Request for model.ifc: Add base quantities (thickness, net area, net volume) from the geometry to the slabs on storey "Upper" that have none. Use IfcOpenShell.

First a look at what the model holds.

```python
import ifcopenshell
import ifcopenshell.util.element
import ifcopenshell.util.unit

model = ifcopenshell.open("model.ifc")
print(model.schema)
for unit_type in ("LENGTHUNIT", "AREAUNIT", "VOLUMEUNIT"):
    print(unit_type, ifcopenshell.util.unit.calculate_unit_scale(model, unit_type))
storey = next(s for s in model.by_type("IfcBuildingStorey") if s.Name == "Upper")
slabs = [e for e in ifcopenshell.util.element.get_decomposition(storey) if e.is_a("IfcSlab")]
for e in sorted(slabs, key=lambda e: e.id()):
    print(e.id(), e.is_a(), e.Name, list(ifcopenshell.util.element.get_psets(e, qtos_only=True)), sep=" | ")
```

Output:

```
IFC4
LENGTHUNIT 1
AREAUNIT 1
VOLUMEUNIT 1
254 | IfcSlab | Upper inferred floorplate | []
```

```python
import ifcopenshell
import ifcopenshell.api.pset
import ifcopenshell.geom
import ifcopenshell.util.element
import ifcopenshell.util.shape
import ifcopenshell.util.unit

model = ifcopenshell.open("model.ifc")
unit_scale = ifcopenshell.util.unit.calculate_unit_scale(model)
area_scale = ifcopenshell.util.unit.calculate_unit_scale(model, "AREAUNIT")
volume_scale = ifcopenshell.util.unit.calculate_unit_scale(model, "VOLUMEUNIT")
settings = ifcopenshell.geom.settings()

storey = next(s for s in model.by_type("IfcBuildingStorey") if s.Name == "Upper")
slabs = [e for e in ifcopenshell.util.element.get_decomposition(storey) if e.is_a("IfcSlab")]

for e in sorted(slabs, key=lambda e: e.id()):
    if ifcopenshell.util.element.get_psets(e, qtos_only=True, should_inherit=False):
        continue
    # Geometry comes back in metres, in the element's own axes.
    shape = ifcopenshell.geom.create_shape(settings, e)
    values = {
        "Width": ifcopenshell.util.shape.get_z(shape.geometry) / unit_scale,
        "NetArea": ifcopenshell.util.shape.get_footprint_area(shape.geometry) / area_scale,
        "NetVolume": ifcopenshell.util.shape.get_volume(shape.geometry) / volume_scale,
    }
    qto = ifcopenshell.api.pset.add_qto(model, product=e, name="Qto_SlabBaseQuantities")
    ifcopenshell.api.pset.edit_qto(model, qto=qto, properties=values)
    print(e.id(), {k: round(v, 3) for k, v in values.items()})

model.write("model_rev.ifc")
```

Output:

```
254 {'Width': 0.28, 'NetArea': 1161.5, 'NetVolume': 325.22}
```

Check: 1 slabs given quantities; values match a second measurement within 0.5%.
